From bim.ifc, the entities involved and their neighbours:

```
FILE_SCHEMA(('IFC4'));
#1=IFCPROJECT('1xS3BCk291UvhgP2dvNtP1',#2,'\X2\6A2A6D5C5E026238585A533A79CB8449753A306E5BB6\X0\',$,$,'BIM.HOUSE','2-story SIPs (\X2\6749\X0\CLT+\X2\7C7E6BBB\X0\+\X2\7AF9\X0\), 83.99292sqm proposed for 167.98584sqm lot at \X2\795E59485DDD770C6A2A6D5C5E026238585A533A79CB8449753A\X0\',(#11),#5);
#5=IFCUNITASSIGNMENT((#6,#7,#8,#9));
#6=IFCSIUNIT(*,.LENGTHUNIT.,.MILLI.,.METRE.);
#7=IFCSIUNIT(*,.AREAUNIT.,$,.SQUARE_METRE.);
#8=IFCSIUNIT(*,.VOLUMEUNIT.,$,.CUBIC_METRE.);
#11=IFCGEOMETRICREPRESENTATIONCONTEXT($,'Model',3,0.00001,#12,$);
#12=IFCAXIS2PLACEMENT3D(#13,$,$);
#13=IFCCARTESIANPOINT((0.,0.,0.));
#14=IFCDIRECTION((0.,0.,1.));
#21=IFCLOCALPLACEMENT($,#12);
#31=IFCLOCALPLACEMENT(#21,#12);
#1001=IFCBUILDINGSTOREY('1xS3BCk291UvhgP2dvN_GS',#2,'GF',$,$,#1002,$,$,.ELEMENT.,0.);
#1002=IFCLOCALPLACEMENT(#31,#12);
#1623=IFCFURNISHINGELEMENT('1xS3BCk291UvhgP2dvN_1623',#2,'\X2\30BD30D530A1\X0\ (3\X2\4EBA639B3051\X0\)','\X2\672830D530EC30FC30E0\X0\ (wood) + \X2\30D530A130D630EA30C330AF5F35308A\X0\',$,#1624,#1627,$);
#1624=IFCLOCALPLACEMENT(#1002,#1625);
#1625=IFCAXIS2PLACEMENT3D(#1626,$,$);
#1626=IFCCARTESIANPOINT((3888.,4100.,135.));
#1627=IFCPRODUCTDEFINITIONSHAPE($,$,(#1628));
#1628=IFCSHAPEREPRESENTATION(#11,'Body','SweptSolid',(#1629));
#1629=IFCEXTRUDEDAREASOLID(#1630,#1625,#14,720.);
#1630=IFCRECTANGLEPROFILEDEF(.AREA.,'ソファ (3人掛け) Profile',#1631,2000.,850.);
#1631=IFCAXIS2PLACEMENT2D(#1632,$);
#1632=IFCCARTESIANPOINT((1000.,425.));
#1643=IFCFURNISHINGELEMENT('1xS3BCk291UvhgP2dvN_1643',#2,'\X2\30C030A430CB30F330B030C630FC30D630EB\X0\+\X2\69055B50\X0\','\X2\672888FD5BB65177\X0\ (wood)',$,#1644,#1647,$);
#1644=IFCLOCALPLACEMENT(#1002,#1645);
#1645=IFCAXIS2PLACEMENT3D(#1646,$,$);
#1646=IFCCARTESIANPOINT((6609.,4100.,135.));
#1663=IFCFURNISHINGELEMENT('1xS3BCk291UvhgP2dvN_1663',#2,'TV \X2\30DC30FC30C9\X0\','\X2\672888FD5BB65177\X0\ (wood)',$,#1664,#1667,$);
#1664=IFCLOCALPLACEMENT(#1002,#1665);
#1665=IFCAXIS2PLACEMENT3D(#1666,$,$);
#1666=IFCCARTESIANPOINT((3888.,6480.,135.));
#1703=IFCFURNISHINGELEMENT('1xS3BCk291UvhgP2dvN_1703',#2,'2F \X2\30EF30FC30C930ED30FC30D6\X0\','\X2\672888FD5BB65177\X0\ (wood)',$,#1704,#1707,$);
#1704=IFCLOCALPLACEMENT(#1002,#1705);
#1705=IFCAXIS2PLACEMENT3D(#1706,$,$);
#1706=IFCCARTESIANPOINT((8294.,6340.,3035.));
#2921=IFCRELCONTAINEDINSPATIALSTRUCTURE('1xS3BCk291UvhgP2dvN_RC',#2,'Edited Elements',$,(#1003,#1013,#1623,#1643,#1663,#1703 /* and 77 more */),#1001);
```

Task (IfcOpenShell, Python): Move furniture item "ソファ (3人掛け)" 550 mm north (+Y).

```python
import ifcopenshell
import ifcopenshell.api.geometry
import ifcopenshell.util.placement
import ifcopenshell.util.unit

model = ifcopenshell.open("bim.ifc")
unit_scale = ifcopenshell.util.unit.calculate_unit_scale(model)

item = model.by_id(1623)
matrix = ifcopenshell.util.placement.get_local_placement(item.ObjectPlacement)
matrix[1, 3] += 0.55 / unit_scale
ifcopenshell.api.geometry.edit_object_placement(model, product=item, matrix=matrix, is_si=False)

print(ifcopenshell.util.placement.get_local_placement(item.ObjectPlacement).round(3) + 0.0)

model.write("bim_rev.ifc")
```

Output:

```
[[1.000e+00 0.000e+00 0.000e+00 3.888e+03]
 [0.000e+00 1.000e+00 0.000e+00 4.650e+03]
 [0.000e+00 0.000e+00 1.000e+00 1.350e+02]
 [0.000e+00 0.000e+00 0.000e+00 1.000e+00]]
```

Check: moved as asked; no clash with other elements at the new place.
